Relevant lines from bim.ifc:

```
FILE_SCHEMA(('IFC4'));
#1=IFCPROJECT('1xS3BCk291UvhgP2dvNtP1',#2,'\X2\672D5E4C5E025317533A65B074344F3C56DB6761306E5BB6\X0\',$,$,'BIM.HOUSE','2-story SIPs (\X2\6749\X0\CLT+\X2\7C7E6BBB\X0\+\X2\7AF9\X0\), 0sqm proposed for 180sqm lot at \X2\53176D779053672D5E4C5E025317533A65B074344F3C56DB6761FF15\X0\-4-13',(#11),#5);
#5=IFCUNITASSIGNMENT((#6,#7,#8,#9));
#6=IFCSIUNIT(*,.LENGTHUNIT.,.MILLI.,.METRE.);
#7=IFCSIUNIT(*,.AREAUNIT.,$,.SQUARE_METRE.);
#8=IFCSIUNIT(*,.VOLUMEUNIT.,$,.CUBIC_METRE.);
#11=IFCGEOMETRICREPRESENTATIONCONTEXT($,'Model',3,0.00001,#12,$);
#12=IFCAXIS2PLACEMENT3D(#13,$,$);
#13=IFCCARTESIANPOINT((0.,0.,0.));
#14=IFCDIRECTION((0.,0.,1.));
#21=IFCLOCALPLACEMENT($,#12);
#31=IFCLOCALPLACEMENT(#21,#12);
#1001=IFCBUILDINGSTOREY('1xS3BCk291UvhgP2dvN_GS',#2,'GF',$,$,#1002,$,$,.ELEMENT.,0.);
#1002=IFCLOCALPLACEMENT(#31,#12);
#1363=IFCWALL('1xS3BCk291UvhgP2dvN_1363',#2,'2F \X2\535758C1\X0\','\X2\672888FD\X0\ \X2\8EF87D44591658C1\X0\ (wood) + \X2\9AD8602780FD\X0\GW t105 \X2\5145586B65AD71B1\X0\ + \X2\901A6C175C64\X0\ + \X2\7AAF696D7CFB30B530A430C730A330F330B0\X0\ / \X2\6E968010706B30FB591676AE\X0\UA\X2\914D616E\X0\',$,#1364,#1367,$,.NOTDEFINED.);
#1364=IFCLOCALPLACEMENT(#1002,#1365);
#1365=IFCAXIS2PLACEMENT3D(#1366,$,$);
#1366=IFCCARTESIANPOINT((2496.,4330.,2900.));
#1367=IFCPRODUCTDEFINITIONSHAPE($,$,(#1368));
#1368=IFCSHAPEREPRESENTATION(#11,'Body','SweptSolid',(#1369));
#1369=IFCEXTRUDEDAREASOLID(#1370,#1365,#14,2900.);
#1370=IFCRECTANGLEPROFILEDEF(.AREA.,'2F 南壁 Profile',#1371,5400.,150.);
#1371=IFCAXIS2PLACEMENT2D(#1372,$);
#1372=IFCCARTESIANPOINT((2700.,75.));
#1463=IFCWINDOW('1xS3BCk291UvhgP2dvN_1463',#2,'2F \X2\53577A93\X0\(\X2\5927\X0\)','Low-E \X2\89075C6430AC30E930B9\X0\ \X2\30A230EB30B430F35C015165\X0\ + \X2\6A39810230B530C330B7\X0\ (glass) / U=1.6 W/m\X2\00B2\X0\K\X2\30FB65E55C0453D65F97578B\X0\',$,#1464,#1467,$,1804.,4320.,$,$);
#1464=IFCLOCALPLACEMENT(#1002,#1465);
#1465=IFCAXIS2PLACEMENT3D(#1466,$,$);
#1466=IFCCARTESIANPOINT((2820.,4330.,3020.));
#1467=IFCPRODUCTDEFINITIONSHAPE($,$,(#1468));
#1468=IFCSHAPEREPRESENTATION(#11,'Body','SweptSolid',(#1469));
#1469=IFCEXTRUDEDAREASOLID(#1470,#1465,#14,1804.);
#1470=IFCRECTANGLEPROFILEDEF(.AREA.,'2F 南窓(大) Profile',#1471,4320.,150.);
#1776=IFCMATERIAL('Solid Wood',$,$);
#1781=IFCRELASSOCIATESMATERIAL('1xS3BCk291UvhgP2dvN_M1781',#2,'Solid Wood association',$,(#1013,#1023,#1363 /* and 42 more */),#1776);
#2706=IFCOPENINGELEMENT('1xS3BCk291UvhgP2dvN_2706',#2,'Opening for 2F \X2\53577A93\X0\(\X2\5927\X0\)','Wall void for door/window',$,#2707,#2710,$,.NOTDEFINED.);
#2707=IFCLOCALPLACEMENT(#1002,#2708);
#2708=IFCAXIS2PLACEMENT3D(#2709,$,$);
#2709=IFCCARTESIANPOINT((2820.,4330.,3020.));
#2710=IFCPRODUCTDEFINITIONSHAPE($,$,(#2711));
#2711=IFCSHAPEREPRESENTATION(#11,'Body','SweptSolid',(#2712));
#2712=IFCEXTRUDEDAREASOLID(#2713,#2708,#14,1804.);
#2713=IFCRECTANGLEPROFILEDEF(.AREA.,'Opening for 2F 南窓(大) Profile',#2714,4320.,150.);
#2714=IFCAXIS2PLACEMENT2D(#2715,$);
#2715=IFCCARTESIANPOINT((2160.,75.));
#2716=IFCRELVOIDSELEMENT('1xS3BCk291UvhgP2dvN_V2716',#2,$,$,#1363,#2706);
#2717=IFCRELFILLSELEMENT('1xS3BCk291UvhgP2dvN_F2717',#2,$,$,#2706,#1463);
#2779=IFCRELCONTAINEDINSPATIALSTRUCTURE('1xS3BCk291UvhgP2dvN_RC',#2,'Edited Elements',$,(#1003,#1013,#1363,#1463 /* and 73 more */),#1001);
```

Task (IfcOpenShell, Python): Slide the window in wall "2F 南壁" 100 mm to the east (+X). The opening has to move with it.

```python
import ifcopenshell
import ifcopenshell.api.geometry
import ifcopenshell.util.placement
import ifcopenshell.util.unit

model = ifcopenshell.open("bim.ifc")
unit_scale = ifcopenshell.util.unit.calculate_unit_scale(model)

window = model.by_guid("1xS3BCk291UvhgP2dvN_1463")
opening = window.FillsVoids[0].RelatingOpeningElement
wall = opening.VoidsElements[0].RelatingBuildingElement

wall_matrix = ifcopenshell.util.placement.get_local_placement(wall.ObjectPlacement)
shift = wall_matrix[:3, 0] * 0.1 / unit_scale
before = ifcopenshell.util.placement.get_local_placement(window.ObjectPlacement)[:3, 3].copy()

# The window is not placed relative to its opening, so move both.
for product in (opening, window):
    matrix = ifcopenshell.util.placement.get_local_placement(product.ObjectPlacement)
    matrix[:3, 3] += shift
    ifcopenshell.api.geometry.edit_object_placement(model, product=product, matrix=matrix, is_si=False)

after = ifcopenshell.util.placement.get_local_placement(window.ObjectPlacement)[:3, 3]
print("window moved by", (after - before).round(3) + 0.0)

model.write("bim_edited.ifc")
```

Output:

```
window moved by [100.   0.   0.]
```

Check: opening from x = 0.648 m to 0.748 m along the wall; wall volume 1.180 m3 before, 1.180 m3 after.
